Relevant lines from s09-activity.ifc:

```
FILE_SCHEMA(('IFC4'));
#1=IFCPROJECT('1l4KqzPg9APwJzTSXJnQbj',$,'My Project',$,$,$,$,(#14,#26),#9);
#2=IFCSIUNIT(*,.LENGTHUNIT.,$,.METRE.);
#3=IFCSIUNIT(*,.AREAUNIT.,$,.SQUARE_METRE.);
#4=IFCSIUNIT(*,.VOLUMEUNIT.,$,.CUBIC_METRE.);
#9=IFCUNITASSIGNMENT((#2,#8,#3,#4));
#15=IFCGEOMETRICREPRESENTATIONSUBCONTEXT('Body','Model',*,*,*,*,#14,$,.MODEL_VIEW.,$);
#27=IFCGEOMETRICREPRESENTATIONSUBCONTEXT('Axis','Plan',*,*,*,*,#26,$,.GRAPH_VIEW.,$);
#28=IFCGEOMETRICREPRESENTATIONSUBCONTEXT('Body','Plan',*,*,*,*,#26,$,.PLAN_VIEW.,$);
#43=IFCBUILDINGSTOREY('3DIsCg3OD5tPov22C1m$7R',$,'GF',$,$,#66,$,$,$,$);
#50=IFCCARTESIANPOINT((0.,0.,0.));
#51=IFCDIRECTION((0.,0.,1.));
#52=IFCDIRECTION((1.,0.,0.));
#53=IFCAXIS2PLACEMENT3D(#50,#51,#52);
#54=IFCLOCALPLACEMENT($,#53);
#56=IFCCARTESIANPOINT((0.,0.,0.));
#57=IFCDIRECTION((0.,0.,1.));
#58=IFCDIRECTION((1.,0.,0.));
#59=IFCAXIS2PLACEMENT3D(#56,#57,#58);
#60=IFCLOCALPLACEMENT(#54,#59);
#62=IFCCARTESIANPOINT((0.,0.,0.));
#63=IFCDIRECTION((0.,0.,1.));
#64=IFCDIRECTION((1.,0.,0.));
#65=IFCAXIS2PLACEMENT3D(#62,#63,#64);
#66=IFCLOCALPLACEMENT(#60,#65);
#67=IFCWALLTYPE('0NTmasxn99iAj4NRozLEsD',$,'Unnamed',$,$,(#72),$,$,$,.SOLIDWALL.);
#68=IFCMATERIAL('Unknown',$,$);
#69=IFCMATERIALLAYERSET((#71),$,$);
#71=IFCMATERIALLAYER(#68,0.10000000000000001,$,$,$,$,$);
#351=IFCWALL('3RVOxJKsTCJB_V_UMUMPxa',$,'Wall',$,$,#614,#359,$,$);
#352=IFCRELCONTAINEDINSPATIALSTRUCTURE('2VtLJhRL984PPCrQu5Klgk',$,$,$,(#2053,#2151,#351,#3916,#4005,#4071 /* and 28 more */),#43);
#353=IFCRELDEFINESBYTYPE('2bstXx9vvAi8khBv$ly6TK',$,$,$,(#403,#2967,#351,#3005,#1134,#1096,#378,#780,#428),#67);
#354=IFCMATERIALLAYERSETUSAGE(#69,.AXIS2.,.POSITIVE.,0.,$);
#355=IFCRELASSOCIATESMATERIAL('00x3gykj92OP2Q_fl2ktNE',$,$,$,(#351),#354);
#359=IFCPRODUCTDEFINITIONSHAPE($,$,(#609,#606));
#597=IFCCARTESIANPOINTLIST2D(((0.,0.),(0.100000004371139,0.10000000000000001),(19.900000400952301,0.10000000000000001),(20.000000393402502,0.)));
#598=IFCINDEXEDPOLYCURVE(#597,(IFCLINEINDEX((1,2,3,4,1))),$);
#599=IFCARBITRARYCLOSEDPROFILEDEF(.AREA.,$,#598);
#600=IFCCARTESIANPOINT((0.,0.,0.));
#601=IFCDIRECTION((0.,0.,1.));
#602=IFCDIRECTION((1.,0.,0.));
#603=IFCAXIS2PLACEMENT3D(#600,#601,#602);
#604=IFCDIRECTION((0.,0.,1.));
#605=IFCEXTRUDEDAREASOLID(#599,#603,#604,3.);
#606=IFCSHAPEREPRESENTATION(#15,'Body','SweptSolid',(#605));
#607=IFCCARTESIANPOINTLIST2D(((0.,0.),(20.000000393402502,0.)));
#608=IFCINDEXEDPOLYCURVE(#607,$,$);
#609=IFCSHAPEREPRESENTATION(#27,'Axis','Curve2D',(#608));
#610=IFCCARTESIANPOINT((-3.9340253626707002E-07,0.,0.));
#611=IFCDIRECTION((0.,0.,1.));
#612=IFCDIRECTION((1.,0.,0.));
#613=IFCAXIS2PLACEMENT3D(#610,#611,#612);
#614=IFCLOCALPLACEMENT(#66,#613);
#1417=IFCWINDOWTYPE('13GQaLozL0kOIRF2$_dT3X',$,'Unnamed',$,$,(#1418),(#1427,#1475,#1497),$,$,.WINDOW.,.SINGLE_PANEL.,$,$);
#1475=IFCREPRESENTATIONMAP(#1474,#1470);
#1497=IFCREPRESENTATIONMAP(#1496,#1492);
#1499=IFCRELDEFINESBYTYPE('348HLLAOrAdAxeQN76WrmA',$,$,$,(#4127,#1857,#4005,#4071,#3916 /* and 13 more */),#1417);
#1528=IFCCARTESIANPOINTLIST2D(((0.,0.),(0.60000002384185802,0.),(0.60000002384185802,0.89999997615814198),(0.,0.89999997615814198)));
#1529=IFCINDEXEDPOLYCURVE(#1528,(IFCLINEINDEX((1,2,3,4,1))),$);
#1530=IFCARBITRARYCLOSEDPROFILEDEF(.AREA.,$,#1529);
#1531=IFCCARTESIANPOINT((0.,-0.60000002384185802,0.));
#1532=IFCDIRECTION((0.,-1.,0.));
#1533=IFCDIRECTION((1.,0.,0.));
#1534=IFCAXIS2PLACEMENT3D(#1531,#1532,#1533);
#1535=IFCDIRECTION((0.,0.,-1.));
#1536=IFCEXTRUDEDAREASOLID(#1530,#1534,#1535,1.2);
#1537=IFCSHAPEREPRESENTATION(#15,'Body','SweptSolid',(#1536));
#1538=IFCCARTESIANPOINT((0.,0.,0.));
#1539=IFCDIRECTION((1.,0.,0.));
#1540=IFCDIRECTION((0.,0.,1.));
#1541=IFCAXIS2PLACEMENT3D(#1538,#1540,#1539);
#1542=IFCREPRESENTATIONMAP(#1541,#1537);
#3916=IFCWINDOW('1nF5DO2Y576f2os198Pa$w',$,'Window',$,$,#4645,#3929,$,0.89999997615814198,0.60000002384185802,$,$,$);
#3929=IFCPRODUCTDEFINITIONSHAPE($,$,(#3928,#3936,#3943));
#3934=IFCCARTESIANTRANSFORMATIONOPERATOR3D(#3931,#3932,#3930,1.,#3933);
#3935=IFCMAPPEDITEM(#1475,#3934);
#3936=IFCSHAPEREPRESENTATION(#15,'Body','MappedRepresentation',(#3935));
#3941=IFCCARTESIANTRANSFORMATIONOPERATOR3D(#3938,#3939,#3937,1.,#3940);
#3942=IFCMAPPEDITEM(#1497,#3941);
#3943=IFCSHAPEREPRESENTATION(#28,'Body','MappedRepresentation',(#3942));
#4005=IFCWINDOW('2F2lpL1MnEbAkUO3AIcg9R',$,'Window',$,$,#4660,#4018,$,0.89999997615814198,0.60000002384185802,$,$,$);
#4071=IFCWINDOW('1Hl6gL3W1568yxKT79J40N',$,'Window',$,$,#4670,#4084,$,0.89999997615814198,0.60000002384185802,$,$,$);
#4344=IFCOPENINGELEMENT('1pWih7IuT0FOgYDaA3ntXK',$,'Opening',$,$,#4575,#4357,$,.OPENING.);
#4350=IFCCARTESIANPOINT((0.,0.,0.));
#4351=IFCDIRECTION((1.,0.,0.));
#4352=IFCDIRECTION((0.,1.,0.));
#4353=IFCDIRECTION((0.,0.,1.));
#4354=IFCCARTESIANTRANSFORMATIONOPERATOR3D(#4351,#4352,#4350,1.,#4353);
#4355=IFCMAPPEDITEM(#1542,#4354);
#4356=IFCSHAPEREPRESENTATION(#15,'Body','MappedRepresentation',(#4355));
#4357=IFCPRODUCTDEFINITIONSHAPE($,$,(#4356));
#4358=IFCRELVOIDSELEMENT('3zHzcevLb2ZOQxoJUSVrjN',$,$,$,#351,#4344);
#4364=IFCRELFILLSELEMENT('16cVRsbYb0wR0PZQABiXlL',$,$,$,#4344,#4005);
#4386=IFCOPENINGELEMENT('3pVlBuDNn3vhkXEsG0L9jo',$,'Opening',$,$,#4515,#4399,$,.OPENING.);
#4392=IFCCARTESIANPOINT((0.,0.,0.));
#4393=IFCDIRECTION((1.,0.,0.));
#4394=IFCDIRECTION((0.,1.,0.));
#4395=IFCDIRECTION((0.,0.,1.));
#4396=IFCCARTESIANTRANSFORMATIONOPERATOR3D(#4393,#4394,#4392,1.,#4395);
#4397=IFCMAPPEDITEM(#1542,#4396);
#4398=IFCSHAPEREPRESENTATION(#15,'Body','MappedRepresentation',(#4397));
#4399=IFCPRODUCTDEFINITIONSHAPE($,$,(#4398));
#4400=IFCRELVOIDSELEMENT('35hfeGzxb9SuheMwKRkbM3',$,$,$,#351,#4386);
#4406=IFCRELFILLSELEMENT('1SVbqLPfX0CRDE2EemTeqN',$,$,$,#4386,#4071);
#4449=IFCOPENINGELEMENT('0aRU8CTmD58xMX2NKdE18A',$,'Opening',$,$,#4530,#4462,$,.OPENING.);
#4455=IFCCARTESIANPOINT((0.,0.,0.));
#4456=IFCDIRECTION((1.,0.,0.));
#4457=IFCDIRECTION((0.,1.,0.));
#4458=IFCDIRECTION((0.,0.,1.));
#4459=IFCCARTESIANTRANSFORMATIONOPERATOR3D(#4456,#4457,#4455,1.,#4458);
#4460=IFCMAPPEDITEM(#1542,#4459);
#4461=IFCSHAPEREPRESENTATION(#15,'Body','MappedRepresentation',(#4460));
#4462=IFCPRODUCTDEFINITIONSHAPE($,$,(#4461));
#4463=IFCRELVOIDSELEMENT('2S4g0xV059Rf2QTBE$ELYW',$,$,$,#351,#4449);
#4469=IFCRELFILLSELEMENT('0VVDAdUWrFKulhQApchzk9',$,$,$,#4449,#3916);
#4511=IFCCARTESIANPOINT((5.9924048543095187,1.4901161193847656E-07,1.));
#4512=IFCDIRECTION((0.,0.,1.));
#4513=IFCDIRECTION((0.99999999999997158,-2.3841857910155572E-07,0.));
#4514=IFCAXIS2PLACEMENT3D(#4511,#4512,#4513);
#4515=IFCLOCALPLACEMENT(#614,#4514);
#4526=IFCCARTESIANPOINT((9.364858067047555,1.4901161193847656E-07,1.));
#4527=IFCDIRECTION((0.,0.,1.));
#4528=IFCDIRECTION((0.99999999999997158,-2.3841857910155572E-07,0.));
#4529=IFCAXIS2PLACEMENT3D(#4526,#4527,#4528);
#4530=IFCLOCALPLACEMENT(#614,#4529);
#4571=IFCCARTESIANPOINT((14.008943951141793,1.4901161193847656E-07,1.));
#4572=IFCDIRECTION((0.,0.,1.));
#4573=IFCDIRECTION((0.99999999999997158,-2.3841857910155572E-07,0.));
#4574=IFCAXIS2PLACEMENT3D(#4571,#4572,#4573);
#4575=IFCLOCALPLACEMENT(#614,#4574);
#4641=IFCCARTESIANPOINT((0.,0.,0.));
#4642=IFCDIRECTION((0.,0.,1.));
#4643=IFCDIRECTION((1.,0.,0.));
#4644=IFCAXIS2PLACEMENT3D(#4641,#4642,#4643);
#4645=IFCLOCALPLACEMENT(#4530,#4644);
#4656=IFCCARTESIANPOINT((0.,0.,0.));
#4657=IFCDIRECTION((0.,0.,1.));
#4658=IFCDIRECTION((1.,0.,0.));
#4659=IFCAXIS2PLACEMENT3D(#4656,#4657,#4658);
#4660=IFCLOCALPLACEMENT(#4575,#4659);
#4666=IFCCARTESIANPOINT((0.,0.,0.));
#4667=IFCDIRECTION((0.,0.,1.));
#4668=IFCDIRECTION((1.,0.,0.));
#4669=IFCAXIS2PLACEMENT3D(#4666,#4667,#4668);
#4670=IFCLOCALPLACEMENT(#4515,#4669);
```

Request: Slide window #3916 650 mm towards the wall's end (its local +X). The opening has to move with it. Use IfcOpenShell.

```python
import ifcopenshell
import ifcopenshell.api.geometry
import ifcopenshell.util.placement
import ifcopenshell.util.unit

model = ifcopenshell.open("s09-activity.ifc")
unit_scale = ifcopenshell.util.unit.calculate_unit_scale(model)

window = model.by_guid("1nF5DO2Y576f2os198Pa$w")
opening = window.FillsVoids[0].RelatingOpeningElement
wall = opening.VoidsElements[0].RelatingBuildingElement

wall_matrix = ifcopenshell.util.placement.get_local_placement(wall.ObjectPlacement)
shift = wall_matrix[:3, 0] * 0.65 / unit_scale
before = ifcopenshell.util.placement.get_local_placement(window.ObjectPlacement)[:3, 3].copy()

# The window is placed relative to its opening, so it follows when the opening moves.
matrix = ifcopenshell.util.placement.get_local_placement(opening.ObjectPlacement)
matrix[:3, 3] += shift
ifcopenshell.api.geometry.edit_object_placement(
    model, product=opening, matrix=matrix, is_si=False, should_transform_children=True
)

after = ifcopenshell.util.placement.get_local_placement(window.ObjectPlacement)[:3, 3]
print("window moved by", (after - before).round(3) + 0.0)

model.write("s09-activity_rev.ifc")
```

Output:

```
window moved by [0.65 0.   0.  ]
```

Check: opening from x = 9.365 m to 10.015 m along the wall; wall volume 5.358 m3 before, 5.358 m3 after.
